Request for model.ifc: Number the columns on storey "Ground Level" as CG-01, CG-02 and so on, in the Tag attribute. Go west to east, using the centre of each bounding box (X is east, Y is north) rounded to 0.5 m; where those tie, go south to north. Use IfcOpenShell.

First a look at what the model holds.

```python
import ifcopenshell
import ifcopenshell.util.element
import ifcopenshell.util.placement

model = ifcopenshell.open("model.ifc")
print(model.schema)
storey = next(s for s in model.by_type("IfcBuildingStorey") if s.Name == "Ground Level")
columns = [e for e in ifcopenshell.util.element.get_decomposition(storey) if e.is_a("IfcColumn")]
for e in sorted(columns, key=lambda e: e.id()):
    origin = ifcopenshell.util.placement.get_local_placement(e.ObjectPlacement)[:3, 3]
    print(e.id(), e.Tag, e.Name, origin.round(2) + 0.0, sep=" | ")
```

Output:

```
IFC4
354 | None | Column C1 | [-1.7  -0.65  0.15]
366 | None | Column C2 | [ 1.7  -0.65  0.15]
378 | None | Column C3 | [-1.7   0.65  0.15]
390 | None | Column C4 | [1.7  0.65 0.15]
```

```python
import ifcopenshell
import ifcopenshell.geom
import ifcopenshell.util.element
import ifcopenshell.util.shape

model = ifcopenshell.open("model.ifc")
settings = ifcopenshell.geom.settings()
settings.set("use-world-coords", True)


def centre(element):
    shape = ifcopenshell.geom.create_shape(settings, element)
    return ifcopenshell.util.shape.get_bbox_centroid(shape.geometry)


storey = next(s for s in model.by_type("IfcBuildingStorey") if s.Name == "Ground Level")
columns = [e for e in ifcopenshell.util.element.get_decomposition(storey) if e.is_a("IfcColumn")]

# Insertion points can sit at a corner or the storey origin, so sort by the geometry (in metres).
centres = {e: centre(e) for e in columns}
columns.sort(key=lambda e: (round(centres[e][0] / 0.5), centres[e][1]))

for i, e in enumerate(columns, start=1):
    number = f"CG-{i:02d}"
    e.Tag = number
    print(e.id(), number)

model.write("model_v2.ifc")
```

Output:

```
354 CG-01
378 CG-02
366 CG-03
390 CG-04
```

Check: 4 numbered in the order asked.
